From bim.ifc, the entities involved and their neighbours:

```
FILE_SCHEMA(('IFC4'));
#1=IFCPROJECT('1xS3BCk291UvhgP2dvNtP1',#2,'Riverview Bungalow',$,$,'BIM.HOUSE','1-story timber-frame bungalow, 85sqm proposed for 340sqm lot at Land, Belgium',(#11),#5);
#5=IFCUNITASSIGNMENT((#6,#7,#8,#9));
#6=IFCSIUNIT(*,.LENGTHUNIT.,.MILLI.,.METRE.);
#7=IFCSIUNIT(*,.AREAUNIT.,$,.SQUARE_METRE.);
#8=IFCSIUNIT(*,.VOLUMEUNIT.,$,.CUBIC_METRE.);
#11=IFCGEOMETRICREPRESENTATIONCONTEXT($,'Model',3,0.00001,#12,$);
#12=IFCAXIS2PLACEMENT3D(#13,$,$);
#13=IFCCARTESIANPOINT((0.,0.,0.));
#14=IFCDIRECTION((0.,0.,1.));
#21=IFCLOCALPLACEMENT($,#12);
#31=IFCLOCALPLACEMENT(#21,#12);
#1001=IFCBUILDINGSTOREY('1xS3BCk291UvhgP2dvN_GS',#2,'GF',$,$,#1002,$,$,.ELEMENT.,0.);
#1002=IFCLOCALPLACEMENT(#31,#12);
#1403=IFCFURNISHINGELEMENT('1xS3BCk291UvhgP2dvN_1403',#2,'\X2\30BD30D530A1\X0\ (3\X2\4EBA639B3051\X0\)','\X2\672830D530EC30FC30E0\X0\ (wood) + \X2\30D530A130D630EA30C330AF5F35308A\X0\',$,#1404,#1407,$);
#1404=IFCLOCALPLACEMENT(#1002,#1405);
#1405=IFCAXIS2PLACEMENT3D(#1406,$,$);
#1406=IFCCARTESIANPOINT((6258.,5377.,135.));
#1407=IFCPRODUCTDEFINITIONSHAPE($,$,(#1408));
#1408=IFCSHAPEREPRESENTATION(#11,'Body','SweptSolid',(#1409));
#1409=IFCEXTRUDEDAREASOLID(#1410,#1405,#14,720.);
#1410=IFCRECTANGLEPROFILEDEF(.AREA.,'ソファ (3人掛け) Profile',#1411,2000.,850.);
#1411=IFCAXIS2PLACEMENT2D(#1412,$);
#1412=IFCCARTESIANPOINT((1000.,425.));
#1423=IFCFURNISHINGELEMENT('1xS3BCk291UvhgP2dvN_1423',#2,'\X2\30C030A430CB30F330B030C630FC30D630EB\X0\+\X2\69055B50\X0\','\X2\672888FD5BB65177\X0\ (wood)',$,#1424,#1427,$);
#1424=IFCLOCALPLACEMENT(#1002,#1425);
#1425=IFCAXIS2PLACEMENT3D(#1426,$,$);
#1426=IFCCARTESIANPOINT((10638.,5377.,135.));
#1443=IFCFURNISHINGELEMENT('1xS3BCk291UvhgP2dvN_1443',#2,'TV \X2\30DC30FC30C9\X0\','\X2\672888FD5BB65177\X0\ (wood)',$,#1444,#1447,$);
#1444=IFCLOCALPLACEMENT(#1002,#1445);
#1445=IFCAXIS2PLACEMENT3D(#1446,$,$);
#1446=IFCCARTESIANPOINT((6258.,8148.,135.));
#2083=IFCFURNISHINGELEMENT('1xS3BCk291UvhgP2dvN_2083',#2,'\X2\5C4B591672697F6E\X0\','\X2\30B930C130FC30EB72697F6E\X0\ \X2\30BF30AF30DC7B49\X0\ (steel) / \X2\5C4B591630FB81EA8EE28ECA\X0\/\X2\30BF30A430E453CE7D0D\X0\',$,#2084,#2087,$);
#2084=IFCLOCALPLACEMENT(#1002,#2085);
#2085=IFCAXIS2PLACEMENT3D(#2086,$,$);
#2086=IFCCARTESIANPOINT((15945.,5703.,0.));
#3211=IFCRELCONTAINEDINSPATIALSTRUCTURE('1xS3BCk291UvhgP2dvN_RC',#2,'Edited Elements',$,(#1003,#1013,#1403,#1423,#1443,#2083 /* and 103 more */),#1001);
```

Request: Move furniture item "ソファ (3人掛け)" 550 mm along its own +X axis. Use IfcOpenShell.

```python
import ifcopenshell
import ifcopenshell.api.geometry
import ifcopenshell.util.placement
import ifcopenshell.util.unit

model = ifcopenshell.open("bim.ifc")
unit_scale = ifcopenshell.util.unit.calculate_unit_scale(model)

item = model.by_guid("1xS3BCk291UvhgP2dvN_1403")
matrix = ifcopenshell.util.placement.get_local_placement(item.ObjectPlacement)
matrix[:3, 3] += matrix[:3, 0] * 0.55 / unit_scale
ifcopenshell.api.geometry.edit_object_placement(model, product=item, matrix=matrix, is_si=False)

print(ifcopenshell.util.placement.get_local_placement(item.ObjectPlacement).round(3) + 0.0)

model.write("bim_rev.ifc")
```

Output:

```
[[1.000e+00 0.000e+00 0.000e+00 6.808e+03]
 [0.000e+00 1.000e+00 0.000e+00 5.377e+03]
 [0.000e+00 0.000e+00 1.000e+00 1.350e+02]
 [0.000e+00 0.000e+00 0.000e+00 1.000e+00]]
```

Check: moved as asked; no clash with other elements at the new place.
